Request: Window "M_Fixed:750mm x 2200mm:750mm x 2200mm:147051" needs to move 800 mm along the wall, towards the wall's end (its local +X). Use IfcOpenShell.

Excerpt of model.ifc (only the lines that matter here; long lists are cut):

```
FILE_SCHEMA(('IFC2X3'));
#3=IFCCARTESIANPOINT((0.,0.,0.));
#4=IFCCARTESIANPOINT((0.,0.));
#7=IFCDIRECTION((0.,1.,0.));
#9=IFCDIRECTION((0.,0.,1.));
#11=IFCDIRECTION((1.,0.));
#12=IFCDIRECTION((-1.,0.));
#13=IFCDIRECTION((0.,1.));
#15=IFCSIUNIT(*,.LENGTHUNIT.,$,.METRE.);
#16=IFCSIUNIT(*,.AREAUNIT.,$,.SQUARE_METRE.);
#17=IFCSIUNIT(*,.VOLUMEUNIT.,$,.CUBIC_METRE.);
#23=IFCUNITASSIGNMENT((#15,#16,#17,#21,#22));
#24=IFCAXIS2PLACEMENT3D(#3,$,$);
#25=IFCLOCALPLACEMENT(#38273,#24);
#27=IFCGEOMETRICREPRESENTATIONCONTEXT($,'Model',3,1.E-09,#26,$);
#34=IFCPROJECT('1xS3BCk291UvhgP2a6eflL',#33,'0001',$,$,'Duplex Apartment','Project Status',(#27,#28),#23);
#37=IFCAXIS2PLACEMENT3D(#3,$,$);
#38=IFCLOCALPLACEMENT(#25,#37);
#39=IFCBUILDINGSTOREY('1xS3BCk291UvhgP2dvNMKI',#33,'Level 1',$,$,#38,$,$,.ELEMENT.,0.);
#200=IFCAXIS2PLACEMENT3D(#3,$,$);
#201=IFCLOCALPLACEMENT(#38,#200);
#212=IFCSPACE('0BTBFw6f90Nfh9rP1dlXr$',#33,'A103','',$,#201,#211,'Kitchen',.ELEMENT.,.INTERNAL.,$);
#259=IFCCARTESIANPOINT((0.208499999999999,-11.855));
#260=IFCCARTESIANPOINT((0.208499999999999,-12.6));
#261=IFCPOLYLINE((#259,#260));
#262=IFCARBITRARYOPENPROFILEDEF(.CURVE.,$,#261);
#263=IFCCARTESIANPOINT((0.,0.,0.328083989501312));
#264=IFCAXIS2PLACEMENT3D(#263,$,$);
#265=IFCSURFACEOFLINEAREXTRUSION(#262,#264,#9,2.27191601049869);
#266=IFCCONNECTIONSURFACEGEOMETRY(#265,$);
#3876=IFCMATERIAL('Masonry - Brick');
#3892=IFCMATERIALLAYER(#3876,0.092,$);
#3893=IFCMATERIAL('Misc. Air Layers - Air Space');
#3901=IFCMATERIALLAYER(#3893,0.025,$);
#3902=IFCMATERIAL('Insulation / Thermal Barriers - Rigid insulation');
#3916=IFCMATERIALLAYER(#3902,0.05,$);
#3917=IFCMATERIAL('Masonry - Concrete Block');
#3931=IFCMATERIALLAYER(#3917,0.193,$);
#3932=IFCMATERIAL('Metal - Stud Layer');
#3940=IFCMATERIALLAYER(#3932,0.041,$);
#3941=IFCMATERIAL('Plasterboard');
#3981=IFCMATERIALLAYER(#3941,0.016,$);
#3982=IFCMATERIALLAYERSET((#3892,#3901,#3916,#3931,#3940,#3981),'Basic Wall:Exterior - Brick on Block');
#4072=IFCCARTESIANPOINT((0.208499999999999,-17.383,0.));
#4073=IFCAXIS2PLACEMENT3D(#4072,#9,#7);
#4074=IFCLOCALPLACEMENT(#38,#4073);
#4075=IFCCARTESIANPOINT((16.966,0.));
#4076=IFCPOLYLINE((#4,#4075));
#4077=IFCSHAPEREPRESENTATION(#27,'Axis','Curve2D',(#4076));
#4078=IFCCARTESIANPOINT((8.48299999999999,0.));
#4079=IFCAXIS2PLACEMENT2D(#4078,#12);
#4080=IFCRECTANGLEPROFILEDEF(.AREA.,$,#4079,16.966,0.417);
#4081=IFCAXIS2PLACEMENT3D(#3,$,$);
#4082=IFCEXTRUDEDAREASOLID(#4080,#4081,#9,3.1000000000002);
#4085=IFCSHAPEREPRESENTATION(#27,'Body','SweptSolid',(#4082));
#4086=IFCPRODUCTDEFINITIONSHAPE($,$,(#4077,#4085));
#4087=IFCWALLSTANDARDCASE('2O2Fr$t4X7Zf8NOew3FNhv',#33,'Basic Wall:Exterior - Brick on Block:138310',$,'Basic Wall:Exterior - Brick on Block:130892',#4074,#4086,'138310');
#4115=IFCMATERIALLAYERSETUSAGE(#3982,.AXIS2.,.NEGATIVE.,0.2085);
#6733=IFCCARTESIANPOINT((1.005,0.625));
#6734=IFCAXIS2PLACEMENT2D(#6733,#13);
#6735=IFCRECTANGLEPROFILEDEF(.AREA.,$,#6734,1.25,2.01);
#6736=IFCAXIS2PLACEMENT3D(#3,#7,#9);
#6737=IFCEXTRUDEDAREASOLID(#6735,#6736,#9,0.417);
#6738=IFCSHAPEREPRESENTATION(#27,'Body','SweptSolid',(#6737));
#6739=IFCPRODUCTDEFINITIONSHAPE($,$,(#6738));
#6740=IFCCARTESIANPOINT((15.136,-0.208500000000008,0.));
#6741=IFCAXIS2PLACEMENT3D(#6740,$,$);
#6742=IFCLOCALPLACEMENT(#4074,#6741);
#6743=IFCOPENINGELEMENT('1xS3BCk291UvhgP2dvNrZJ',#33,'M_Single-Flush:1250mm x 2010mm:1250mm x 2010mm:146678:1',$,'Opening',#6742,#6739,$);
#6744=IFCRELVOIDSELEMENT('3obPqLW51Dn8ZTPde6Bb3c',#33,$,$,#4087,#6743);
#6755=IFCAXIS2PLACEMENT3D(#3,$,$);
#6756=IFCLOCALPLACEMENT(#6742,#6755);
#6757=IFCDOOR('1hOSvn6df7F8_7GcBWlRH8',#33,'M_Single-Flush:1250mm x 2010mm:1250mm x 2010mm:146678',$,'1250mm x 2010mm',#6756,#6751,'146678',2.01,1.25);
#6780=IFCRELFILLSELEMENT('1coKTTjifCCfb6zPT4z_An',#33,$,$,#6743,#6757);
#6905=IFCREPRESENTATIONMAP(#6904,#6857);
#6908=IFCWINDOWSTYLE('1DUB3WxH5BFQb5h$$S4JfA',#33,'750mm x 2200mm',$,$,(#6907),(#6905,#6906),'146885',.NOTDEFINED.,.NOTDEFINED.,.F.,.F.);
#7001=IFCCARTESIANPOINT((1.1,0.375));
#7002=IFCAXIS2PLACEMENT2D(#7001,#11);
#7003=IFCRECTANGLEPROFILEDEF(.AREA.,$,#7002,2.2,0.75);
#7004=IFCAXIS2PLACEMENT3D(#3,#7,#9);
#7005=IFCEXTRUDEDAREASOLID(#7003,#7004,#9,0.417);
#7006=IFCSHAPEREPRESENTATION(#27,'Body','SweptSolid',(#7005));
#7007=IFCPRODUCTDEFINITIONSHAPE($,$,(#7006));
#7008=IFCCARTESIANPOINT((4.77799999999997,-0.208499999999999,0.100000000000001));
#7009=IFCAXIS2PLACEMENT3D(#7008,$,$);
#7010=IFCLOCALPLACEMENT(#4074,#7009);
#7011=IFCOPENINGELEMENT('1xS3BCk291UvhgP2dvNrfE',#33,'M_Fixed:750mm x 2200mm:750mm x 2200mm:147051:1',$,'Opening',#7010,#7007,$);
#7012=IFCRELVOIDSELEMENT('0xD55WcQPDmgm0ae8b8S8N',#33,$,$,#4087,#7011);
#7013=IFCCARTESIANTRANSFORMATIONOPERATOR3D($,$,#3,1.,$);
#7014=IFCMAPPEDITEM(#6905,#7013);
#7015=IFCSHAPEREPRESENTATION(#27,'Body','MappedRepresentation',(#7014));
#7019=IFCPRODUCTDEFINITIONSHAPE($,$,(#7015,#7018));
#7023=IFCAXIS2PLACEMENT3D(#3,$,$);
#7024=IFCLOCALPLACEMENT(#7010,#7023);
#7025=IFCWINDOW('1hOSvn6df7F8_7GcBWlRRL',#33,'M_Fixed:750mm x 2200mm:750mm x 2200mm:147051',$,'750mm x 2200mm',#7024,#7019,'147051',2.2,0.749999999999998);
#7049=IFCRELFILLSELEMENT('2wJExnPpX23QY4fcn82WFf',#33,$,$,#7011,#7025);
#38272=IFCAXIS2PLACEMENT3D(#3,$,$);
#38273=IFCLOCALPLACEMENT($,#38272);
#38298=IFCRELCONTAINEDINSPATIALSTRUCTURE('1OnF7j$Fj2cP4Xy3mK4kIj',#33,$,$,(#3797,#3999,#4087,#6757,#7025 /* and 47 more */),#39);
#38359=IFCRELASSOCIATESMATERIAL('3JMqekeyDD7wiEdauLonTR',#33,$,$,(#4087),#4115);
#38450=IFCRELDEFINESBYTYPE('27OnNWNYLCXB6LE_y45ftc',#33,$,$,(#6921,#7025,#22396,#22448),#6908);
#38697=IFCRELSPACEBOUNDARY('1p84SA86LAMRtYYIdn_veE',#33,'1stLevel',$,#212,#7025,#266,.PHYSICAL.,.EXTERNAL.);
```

```python
import numpy as np
import ifcopenshell
import ifcopenshell.api.geometry
import ifcopenshell.util.placement
import ifcopenshell.util.unit

model = ifcopenshell.open("model.ifc")
unit_scale = ifcopenshell.util.unit.calculate_unit_scale(model)

window = model.by_id(7025)
opening = window.FillsVoids[0].RelatingOpeningElement
wall = opening.VoidsElements[0].RelatingBuildingElement

wall_matrix = ifcopenshell.util.placement.get_local_placement(wall.ObjectPlacement)
shift = wall_matrix[:3, 0] * 0.8 / unit_scale
before = ifcopenshell.util.placement.get_local_placement(window.ObjectPlacement)[:3, 3].copy()

# The window is placed relative to its opening, so it follows when the opening moves.
matrix = ifcopenshell.util.placement.get_local_placement(opening.ObjectPlacement)
matrix[:3, 3] += shift
ifcopenshell.api.geometry.edit_object_placement(
    model, product=opening, matrix=matrix, is_si=False, should_transform_children=True
)

# Space boundary surfaces are stored in each space's coordinates; move them too.
for rel in window.ProvidesBoundaries:
    if not rel.ConnectionGeometry:
        continue
    surface = rel.ConnectionGeometry.SurfaceOnRelatingElement
    space_matrix = ifcopenshell.util.placement.get_local_placement(rel.RelatingSpace.ObjectPlacement)
    point = np.array(surface.Position.Location.Coordinates) + space_matrix[:3, :3].T @ shift
    surface.Position = model.createIfcAxis2Placement3D(
        model.createIfcCartesianPoint(point.tolist()), surface.Position.Axis, surface.Position.RefDirection
    )

after = ifcopenshell.util.placement.get_local_placement(window.ObjectPlacement)[:3, 3]
print("window moved by", (after - before).round(3) + 0.0)

model.write("model_updated.ifc")
```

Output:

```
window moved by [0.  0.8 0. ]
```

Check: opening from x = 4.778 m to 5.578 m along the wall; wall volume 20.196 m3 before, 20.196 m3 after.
